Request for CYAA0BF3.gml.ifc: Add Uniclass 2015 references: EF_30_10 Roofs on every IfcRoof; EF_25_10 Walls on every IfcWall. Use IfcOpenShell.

First a look at what the model holds.

```python
import ifcopenshell

model = ifcopenshell.open("CYAA0BF3.gml.ifc")
print(model.schema)
print("classifications:", [c.Name for c in model.by_type("IfcClassification")])
for ifc_class in ("IfcDoor", "IfcRoof", "IfcStair", "IfcWall", "IfcWindow"):
    print(ifc_class, len(model.by_type(ifc_class)))
```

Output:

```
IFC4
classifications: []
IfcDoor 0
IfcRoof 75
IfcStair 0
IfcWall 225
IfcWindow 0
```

```python
import ifcopenshell
import ifcopenshell.api.classification

model = ifcopenshell.open("CYAA0BF3.gml.ifc")

system = ifcopenshell.api.classification.add_classification(model, classification="Uniclass 2015")

codes = {
    "IfcRoof": ("EF_30_10", "Roofs"),
    "IfcWall": ("EF_25_10", "Walls"),
}
for ifc_class, (code, name) in codes.items():
    products = model.by_type(ifc_class)
    ifcopenshell.api.classification.add_reference(
        model, products=products, classification=system, identification=code, name=name
    )
    print(code, len(products))

model.write("CYAA0BF3.gml_rev.ifc")
```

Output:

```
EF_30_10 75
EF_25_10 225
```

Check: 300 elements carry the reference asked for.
